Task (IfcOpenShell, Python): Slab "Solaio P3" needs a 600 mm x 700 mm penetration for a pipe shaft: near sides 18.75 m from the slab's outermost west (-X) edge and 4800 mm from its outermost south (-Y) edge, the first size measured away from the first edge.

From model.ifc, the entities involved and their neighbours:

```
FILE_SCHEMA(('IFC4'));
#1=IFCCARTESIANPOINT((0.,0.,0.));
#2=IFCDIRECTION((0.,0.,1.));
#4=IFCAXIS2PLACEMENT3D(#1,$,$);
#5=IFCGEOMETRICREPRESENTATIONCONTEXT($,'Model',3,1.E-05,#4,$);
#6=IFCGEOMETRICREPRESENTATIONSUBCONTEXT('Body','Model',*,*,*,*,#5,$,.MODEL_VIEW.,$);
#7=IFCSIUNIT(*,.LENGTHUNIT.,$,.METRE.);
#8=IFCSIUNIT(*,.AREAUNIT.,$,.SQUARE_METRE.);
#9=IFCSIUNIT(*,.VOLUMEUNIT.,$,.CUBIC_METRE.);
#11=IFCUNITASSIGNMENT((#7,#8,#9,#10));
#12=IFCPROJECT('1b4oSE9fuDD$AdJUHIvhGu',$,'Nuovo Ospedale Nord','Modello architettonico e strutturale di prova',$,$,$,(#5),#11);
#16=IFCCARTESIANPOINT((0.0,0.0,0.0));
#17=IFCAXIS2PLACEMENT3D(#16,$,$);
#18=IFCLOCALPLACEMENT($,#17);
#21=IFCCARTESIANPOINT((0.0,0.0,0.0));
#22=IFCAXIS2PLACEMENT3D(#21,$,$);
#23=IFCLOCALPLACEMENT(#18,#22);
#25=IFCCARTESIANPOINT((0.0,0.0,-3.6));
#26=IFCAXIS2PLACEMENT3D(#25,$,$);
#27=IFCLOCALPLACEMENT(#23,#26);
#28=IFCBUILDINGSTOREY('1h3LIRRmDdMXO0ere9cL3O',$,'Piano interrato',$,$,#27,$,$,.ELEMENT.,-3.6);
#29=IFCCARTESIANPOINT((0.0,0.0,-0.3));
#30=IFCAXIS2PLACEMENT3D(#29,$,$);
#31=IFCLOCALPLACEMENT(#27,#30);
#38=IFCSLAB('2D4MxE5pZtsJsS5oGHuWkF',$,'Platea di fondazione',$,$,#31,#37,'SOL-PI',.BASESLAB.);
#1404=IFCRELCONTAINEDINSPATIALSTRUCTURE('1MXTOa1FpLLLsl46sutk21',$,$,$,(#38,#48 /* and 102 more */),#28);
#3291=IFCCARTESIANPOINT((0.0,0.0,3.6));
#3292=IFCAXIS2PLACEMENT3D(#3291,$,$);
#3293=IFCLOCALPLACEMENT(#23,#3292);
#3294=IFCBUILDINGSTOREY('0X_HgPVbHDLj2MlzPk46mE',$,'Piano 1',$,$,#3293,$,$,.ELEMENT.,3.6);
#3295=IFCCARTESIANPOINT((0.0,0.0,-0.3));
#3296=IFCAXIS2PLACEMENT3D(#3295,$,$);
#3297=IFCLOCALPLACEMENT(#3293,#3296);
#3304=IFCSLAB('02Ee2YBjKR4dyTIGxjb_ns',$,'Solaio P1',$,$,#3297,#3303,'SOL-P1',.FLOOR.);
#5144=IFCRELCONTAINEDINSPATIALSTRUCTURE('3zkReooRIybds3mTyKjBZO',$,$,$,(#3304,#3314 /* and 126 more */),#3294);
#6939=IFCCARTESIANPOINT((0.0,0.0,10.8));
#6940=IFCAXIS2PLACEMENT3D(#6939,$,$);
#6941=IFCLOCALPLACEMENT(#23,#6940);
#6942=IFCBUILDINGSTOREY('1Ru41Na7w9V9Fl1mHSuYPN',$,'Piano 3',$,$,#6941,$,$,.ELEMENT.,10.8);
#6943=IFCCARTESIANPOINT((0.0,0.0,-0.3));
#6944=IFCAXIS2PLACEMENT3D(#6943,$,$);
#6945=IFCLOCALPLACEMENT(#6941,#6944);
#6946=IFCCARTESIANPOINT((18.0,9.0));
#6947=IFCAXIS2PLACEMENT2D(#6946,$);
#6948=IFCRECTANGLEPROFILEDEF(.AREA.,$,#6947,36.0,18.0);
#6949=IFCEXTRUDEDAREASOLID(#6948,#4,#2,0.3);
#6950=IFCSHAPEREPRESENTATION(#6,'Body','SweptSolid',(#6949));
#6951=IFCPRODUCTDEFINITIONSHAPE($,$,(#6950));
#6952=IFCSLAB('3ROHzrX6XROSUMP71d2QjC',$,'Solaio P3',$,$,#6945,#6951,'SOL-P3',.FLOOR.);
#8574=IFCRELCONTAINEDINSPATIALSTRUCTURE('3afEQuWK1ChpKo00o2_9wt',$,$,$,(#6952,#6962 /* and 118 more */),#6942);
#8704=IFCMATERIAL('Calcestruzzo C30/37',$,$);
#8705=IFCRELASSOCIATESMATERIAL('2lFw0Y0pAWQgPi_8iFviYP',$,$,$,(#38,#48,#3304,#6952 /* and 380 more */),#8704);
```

```python
import numpy as np
import ifcopenshell
import ifcopenshell.api.feature
import ifcopenshell.api.geometry
import ifcopenshell.api.root
import ifcopenshell.geom
import ifcopenshell.util.placement
import ifcopenshell.util.representation
import ifcopenshell.util.shape
import ifcopenshell.util.unit

model = ifcopenshell.open("model.ifc")
unit_scale = ifcopenshell.util.unit.calculate_unit_scale(model)
settings = ifcopenshell.geom.settings()


def volume(element):
    """Net volume in cubic metres, openings subtracted."""
    shape = ifcopenshell.geom.create_shape(settings, element)
    return ifcopenshell.util.shape.get_volume(shape.geometry)


slab = model.by_id(6952)
before = volume(slab)

# Extent in the slab's own axes, in metres. The edges named are its -X and -Y sides.
slab_shape = ifcopenshell.geom.create_shape(settings, slab)
vertices = ifcopenshell.util.shape.get_vertices(slab_shape.geometry)
x_min, y_min, bottom = vertices.min(axis=0)
top = vertices[:, 2].max()

opening = ifcopenshell.api.root.create_entity(model, ifc_class="IfcOpeningElement", name="Pipe shaft opening", predefined_type="OPENING")
context = ifcopenshell.util.representation.get_context(model, "Model", "Body", "MODEL_VIEW")
width, depth = 0.6, 0.7
outline = [(0.0, 0.0), (width, 0.0), (width, depth), (0.0, depth), (0.0, 0.0)]
# Overshoot both faces by 50 mm so the cut is clean.
shape = ifcopenshell.api.geometry.add_slab_representation(
    model, context=context, depth=top - bottom + 0.1, polyline=outline
)
ifcopenshell.api.geometry.assign_representation(model, product=opening, representation=shape)

matrix = ifcopenshell.util.placement.get_local_placement(slab.ObjectPlacement)
matrix[:, 3] = matrix @ np.append(np.array([x_min + 18.75, y_min + 4.8, bottom - 0.05]) / unit_scale, 1.0)
ifcopenshell.api.geometry.edit_object_placement(model, product=opening, matrix=matrix, is_si=False)
ifcopenshell.api.feature.add_feature(model, feature=opening, element=slab)

after = volume(slab)

print(f"slab volume {before:.3f} -> {after:.3f} m3")

model.write("model-out.ifc")
```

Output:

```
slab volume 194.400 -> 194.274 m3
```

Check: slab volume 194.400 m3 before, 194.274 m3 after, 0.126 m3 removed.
